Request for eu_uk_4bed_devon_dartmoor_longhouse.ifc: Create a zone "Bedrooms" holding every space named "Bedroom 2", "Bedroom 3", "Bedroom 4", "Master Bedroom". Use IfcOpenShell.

First a look at what the model holds.

```python
import ifcopenshell

model = ifcopenshell.open("eu_uk_4bed_devon_dartmoor_longhouse.ifc")
print(model.schema)
seen = {}
for space in model.by_type("IfcSpace"):
    seen[space.LongName] = seen.get(space.LongName, 0) + 1
for name, count in sorted(seen.items(), key=str):
    print(count, "x", name)
print("zones:", [z.Name for z in model.by_type("IfcZone")][:20])
```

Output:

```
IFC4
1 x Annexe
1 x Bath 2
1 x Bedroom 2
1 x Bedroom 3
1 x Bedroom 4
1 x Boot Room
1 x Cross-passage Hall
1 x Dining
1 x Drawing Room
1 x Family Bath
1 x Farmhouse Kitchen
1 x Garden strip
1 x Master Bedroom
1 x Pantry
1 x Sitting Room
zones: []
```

```python
import ifcopenshell
import ifcopenshell.api.group
import ifcopenshell.api.root

model = ifcopenshell.open("eu_uk_4bed_devon_dartmoor_longhouse.ifc")

names = {"Bedroom 2", "Bedroom 3", "Bedroom 4", "Master Bedroom"}
spaces = [s for s in model.by_type("IfcSpace") if s.LongName in names]

zone = ifcopenshell.api.root.create_entity(model, ifc_class="IfcZone", name="Bedrooms")
ifcopenshell.api.group.assign_group(model, products=spaces, group=zone)
print(len(spaces), "spaces in", zone.Name)

model.write("eu_uk_4bed_devon_dartmoor_longhouse_updated.ifc")
```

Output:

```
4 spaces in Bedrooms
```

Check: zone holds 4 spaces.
